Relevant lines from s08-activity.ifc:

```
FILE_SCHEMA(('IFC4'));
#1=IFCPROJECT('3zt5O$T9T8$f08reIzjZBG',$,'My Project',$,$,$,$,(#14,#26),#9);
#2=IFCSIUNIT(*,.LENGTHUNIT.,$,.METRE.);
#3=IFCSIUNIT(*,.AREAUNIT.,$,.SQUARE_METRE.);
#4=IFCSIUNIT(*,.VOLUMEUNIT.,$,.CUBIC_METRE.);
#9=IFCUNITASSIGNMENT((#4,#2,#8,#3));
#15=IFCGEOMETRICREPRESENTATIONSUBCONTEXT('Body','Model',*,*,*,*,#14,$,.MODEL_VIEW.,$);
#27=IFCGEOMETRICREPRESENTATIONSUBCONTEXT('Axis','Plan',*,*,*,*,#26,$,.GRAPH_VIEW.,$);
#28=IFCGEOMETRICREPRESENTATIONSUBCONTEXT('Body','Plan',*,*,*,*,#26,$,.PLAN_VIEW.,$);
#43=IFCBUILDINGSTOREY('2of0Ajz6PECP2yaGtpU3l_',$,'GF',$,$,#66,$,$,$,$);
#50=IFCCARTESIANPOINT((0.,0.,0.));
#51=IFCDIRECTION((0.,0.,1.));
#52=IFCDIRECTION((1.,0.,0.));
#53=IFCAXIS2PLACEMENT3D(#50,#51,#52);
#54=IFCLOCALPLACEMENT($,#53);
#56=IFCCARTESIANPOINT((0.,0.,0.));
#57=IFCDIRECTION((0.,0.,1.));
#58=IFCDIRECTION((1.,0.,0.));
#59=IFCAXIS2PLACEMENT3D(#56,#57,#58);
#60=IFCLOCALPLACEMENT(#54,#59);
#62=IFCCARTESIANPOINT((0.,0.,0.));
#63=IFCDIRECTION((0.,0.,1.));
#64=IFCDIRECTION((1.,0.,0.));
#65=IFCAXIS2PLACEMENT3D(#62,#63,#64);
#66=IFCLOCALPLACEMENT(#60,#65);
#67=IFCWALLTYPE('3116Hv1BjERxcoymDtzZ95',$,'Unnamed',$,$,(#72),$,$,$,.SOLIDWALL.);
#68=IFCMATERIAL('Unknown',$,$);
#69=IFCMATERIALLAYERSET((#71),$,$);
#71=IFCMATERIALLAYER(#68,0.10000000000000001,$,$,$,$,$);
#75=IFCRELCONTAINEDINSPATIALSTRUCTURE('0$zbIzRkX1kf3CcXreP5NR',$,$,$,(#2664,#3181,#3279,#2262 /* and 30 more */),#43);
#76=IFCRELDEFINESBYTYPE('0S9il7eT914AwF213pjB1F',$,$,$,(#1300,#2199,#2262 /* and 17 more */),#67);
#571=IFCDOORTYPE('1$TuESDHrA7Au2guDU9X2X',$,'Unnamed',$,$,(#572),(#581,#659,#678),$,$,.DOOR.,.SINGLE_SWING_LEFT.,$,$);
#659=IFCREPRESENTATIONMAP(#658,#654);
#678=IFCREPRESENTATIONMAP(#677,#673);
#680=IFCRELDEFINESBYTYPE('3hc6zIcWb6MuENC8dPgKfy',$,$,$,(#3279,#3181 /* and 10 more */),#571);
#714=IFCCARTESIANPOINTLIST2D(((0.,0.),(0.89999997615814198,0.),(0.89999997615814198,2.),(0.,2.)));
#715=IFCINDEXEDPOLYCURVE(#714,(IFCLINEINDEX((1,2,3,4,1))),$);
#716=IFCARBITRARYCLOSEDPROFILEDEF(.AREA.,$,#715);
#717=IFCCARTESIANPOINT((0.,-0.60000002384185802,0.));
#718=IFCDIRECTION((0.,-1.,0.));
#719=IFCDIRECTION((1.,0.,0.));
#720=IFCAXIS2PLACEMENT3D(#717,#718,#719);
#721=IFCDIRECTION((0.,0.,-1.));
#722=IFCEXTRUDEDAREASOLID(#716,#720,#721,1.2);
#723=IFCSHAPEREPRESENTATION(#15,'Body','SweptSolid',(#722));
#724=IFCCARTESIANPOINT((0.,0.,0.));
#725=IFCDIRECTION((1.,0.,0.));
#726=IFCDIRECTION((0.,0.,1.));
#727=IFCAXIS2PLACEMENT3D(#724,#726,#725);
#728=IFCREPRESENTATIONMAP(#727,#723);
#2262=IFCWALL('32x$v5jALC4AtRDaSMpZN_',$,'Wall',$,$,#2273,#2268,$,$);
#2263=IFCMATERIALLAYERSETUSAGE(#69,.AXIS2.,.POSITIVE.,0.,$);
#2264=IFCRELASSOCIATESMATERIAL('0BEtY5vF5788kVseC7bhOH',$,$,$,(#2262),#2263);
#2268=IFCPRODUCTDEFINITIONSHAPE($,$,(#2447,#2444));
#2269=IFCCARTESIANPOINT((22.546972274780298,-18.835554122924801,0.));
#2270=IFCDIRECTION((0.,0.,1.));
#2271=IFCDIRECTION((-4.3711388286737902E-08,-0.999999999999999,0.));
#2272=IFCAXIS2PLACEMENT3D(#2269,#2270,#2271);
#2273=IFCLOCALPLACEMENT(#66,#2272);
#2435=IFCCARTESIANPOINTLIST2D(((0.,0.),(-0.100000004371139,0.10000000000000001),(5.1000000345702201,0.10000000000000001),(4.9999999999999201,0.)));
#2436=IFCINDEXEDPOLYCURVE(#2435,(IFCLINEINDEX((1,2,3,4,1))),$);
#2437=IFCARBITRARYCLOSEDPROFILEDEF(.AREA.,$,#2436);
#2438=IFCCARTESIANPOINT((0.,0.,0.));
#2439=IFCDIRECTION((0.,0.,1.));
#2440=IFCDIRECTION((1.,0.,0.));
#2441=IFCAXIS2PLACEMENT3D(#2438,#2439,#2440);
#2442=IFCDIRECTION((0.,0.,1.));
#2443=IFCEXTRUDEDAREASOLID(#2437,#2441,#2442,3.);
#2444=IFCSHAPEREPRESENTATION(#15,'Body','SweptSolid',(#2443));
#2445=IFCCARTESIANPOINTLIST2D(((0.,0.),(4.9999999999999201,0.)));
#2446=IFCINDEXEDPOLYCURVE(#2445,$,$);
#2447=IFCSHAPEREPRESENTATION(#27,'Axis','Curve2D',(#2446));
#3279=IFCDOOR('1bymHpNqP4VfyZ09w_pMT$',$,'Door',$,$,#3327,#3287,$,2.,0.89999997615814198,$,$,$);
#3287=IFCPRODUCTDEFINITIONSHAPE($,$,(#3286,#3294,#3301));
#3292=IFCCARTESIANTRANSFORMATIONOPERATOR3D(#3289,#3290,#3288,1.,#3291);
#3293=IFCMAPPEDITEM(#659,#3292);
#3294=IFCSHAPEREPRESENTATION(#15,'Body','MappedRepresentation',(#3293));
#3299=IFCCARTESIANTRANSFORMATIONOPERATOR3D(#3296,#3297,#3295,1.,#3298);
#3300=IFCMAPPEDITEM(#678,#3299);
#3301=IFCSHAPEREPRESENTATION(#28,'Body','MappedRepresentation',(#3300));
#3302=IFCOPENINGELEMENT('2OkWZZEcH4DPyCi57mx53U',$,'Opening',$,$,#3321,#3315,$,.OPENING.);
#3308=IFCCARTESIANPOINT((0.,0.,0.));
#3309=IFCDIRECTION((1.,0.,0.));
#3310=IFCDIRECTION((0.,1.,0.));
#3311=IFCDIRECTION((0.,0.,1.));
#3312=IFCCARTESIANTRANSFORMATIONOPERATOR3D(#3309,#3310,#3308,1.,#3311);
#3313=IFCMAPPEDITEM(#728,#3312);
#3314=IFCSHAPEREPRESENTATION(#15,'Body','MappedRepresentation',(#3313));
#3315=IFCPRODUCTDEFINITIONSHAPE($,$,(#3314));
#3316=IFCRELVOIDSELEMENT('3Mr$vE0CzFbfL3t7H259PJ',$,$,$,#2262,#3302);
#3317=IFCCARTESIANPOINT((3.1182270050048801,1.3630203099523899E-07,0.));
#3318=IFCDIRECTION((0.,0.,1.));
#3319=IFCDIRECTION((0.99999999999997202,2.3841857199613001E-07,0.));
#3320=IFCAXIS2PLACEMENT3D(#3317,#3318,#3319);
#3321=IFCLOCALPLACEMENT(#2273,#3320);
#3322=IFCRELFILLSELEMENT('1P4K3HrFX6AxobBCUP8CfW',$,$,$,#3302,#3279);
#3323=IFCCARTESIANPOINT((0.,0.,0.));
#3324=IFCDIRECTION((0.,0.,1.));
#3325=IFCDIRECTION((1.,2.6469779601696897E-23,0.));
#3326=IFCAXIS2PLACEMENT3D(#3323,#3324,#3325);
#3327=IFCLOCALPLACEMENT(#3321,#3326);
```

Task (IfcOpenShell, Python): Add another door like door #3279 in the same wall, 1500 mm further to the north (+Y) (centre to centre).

```python
import ifcopenshell
import ifcopenshell.api.feature
import ifcopenshell.api.geometry
import ifcopenshell.api.root
import ifcopenshell.geom
import ifcopenshell.util.element
import ifcopenshell.util.placement
import ifcopenshell.util.shape
import ifcopenshell.util.unit

model = ifcopenshell.open("s08-activity.ifc")
unit_scale = ifcopenshell.util.unit.calculate_unit_scale(model)
settings = ifcopenshell.geom.settings()


def volume(element):
    """Net volume in cubic metres, openings subtracted."""
    shape = ifcopenshell.geom.create_shape(settings, element)
    return ifcopenshell.util.shape.get_volume(shape.geometry)


door = model.by_guid("1bymHpNqP4VfyZ09w_pMT$")
opening = door.FillsVoids[0].RelatingOpeningElement
wall = opening.VoidsElements[0].RelatingBuildingElement
before = volume(wall)
shift = ifcopenshell.util.placement.get_local_placement(wall.ObjectPlacement)[:3, 0] * -1.5 / unit_scale

# copy_class copies the void relationship, type, container and properties, but no geometry.
new_opening = ifcopenshell.api.root.copy_class(model, product=opening)
new_opening.Representation = ifcopenshell.util.element.copy_deep(
    model, opening.Representation, exclude=["IfcGeometricRepresentationContext", "IfcRepresentationMap"]
)
new_door = ifcopenshell.api.root.copy_class(model, product=door)
new_door.Representation = ifcopenshell.util.element.copy_deep(
    model, door.Representation, exclude=["IfcGeometricRepresentationContext", "IfcRepresentationMap"]
)
ifcopenshell.api.feature.add_filling(model, opening=new_opening, element=new_door)

for old, new in ((opening, new_opening), (door, new_door)):
    matrix = ifcopenshell.util.placement.get_local_placement(old.ObjectPlacement)
    matrix[:3, 3] += shift
    ifcopenshell.api.geometry.edit_object_placement(model, product=new, matrix=matrix, is_si=False)

after = volume(wall)

print(f"wall volume {before:.3f} -> {after:.3f} m3")

model.write("s08-activity_rev.ifc")
```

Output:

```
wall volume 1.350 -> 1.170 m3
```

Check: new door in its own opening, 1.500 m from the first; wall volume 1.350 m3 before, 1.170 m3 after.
